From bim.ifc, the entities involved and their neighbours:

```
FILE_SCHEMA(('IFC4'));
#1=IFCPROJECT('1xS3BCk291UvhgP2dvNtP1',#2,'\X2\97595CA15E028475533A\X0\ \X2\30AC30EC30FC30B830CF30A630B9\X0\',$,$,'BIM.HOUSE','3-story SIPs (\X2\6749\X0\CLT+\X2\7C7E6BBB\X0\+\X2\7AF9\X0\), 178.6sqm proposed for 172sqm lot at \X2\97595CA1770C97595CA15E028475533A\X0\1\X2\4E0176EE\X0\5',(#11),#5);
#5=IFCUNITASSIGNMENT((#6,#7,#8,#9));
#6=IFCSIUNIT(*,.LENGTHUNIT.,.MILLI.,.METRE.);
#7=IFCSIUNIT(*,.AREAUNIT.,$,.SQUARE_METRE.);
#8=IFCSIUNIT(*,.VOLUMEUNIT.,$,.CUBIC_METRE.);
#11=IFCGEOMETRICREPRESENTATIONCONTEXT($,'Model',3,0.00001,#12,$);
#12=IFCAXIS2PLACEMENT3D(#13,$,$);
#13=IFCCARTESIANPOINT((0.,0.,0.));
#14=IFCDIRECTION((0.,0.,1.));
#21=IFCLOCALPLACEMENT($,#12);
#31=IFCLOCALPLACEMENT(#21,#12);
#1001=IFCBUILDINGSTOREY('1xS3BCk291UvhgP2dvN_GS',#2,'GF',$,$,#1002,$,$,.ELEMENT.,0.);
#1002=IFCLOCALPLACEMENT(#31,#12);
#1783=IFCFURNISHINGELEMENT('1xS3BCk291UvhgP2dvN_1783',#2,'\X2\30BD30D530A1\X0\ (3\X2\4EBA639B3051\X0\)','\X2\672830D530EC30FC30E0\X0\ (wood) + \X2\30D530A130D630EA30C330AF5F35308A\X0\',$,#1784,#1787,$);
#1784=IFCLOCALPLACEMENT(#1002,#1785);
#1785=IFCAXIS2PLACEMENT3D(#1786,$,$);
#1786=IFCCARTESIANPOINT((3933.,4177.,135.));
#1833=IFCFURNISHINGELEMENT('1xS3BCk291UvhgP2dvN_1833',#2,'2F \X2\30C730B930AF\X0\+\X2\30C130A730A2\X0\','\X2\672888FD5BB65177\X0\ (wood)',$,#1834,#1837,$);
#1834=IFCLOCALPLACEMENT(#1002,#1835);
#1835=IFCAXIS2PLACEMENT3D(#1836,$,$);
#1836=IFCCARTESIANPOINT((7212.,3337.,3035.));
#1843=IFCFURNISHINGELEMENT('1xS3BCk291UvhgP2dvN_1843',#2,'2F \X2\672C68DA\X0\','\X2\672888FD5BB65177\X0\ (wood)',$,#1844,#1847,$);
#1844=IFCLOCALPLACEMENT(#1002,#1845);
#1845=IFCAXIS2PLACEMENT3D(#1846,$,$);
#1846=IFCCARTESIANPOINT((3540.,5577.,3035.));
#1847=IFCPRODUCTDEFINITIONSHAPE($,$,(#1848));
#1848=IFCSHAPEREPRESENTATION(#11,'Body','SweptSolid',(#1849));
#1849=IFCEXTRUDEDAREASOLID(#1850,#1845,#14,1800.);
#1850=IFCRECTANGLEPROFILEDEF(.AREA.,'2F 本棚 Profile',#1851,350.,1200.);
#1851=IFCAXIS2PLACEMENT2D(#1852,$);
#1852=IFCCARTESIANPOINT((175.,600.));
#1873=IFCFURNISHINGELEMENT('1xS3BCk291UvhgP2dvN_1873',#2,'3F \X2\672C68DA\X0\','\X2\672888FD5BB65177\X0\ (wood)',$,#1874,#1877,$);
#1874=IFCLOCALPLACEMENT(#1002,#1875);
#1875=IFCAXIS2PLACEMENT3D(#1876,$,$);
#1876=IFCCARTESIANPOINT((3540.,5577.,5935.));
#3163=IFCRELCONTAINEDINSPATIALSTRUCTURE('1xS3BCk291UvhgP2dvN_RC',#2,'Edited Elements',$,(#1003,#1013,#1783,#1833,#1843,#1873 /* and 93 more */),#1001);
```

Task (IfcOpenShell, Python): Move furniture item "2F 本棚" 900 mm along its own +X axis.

```python
import ifcopenshell
import ifcopenshell.api.geometry
import ifcopenshell.util.placement

model = ifcopenshell.open("bim.ifc")

item = model.by_guid("1xS3BCk291UvhgP2dvN_1843")
matrix = ifcopenshell.util.placement.get_local_placement(item.ObjectPlacement)
matrix[:3, 3] += matrix[:3, 0] * 900.0
ifcopenshell.api.geometry.edit_object_placement(model, product=item, matrix=matrix, is_si=False)

print(ifcopenshell.util.placement.get_local_placement(item.ObjectPlacement).round(3) + 0.0)

model.write("bim_rev.ifc")
```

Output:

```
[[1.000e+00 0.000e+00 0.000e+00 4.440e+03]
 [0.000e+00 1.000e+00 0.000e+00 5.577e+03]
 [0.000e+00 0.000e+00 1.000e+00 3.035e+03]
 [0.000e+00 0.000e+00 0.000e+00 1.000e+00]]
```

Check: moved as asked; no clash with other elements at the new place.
